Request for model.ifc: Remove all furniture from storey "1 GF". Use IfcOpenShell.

First a look at what the model holds.

```python
import ifcopenshell
import ifcopenshell.util.element

model = ifcopenshell.open("model.ifc")
print(model.schema)
storey = next(s for s in model.by_type("IfcBuildingStorey") if s.Name == "1 GF")
furniture = [e for e in ifcopenshell.util.element.get_decomposition(storey) if e.is_a("IfcFurnishingElement")]
seen = {}
for e in furniture:
    element_type = ifcopenshell.util.element.get_type(e)
    name = element_type.Name if element_type not in (None, e) else None
    seen[name] = seen.get(name, 0) + 1
for name, count in sorted(seen.items(), key=str):
    print(count, "x", name)
```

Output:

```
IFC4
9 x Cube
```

```python
import ifcopenshell
import ifcopenshell.api.root
import ifcopenshell.util.element

model = ifcopenshell.open("model.ifc")

storey = next(s for s in model.by_type("IfcBuildingStorey") if s.Name == "1 GF")
furniture = [e for e in ifcopenshell.util.element.get_decomposition(storey) if e.is_a("IfcFurnishingElement")]

for e in furniture:
    ifcopenshell.api.root.remove_product(model, product=e)
print(len(furniture), "removed")

model.write("model_updated.ifc")
```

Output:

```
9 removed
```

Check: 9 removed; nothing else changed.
